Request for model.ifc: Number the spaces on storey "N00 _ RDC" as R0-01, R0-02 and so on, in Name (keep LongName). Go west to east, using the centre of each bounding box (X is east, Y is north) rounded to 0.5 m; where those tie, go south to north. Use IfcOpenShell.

First a look at what the model holds.

```python
import ifcopenshell
import ifcopenshell.util.element
import ifcopenshell.util.placement

model = ifcopenshell.open("model.ifc")
print(model.schema)
storey = next(s for s in model.by_type("IfcBuildingStorey") if s.Name == "N00 _ RDC")
spaces = [e for e in ifcopenshell.util.element.get_decomposition(storey) if e.is_a("IfcSpace")]
for e in sorted(spaces, key=lambda e: e.id()):
    origin = ifcopenshell.util.placement.get_local_placement(e.ObjectPlacement)[:3, 3]
    print(e.id(), e.Name, e.LongName, origin.round(2) + 0.0, sep=" | ")
```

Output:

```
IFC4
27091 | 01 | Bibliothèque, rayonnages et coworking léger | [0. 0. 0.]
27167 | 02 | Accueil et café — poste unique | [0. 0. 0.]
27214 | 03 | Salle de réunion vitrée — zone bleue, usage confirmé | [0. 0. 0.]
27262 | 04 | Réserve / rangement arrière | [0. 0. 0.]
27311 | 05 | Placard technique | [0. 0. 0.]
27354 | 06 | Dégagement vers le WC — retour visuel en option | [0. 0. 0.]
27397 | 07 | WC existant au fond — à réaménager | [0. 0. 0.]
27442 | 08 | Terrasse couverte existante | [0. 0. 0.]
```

```python
import ifcopenshell
import ifcopenshell.geom
import ifcopenshell.util.element
import ifcopenshell.util.shape

model = ifcopenshell.open("model.ifc")
settings = ifcopenshell.geom.settings()
settings.set("use-world-coords", True)


def centre(element):
    shape = ifcopenshell.geom.create_shape(settings, element)
    return ifcopenshell.util.shape.get_bbox_centroid(shape.geometry)


storey = next(s for s in model.by_type("IfcBuildingStorey") if s.Name == "N00 _ RDC")
spaces = [e for e in ifcopenshell.util.element.get_decomposition(storey) if e.is_a("IfcSpace")]

# Insertion points can sit at a corner or the storey origin, so sort by the geometry (in metres).
centres = {e: centre(e) for e in spaces}
spaces.sort(key=lambda e: (round(centres[e][0] / 0.5), centres[e][1]))

for i, e in enumerate(spaces, start=1):
    number = f"R0-{i:02d}"
    e.Name = number
    print(e.id(), number)

model.write("model-out.ifc")
```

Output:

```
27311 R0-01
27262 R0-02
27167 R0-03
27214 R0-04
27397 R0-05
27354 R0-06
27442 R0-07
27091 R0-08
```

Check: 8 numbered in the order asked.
